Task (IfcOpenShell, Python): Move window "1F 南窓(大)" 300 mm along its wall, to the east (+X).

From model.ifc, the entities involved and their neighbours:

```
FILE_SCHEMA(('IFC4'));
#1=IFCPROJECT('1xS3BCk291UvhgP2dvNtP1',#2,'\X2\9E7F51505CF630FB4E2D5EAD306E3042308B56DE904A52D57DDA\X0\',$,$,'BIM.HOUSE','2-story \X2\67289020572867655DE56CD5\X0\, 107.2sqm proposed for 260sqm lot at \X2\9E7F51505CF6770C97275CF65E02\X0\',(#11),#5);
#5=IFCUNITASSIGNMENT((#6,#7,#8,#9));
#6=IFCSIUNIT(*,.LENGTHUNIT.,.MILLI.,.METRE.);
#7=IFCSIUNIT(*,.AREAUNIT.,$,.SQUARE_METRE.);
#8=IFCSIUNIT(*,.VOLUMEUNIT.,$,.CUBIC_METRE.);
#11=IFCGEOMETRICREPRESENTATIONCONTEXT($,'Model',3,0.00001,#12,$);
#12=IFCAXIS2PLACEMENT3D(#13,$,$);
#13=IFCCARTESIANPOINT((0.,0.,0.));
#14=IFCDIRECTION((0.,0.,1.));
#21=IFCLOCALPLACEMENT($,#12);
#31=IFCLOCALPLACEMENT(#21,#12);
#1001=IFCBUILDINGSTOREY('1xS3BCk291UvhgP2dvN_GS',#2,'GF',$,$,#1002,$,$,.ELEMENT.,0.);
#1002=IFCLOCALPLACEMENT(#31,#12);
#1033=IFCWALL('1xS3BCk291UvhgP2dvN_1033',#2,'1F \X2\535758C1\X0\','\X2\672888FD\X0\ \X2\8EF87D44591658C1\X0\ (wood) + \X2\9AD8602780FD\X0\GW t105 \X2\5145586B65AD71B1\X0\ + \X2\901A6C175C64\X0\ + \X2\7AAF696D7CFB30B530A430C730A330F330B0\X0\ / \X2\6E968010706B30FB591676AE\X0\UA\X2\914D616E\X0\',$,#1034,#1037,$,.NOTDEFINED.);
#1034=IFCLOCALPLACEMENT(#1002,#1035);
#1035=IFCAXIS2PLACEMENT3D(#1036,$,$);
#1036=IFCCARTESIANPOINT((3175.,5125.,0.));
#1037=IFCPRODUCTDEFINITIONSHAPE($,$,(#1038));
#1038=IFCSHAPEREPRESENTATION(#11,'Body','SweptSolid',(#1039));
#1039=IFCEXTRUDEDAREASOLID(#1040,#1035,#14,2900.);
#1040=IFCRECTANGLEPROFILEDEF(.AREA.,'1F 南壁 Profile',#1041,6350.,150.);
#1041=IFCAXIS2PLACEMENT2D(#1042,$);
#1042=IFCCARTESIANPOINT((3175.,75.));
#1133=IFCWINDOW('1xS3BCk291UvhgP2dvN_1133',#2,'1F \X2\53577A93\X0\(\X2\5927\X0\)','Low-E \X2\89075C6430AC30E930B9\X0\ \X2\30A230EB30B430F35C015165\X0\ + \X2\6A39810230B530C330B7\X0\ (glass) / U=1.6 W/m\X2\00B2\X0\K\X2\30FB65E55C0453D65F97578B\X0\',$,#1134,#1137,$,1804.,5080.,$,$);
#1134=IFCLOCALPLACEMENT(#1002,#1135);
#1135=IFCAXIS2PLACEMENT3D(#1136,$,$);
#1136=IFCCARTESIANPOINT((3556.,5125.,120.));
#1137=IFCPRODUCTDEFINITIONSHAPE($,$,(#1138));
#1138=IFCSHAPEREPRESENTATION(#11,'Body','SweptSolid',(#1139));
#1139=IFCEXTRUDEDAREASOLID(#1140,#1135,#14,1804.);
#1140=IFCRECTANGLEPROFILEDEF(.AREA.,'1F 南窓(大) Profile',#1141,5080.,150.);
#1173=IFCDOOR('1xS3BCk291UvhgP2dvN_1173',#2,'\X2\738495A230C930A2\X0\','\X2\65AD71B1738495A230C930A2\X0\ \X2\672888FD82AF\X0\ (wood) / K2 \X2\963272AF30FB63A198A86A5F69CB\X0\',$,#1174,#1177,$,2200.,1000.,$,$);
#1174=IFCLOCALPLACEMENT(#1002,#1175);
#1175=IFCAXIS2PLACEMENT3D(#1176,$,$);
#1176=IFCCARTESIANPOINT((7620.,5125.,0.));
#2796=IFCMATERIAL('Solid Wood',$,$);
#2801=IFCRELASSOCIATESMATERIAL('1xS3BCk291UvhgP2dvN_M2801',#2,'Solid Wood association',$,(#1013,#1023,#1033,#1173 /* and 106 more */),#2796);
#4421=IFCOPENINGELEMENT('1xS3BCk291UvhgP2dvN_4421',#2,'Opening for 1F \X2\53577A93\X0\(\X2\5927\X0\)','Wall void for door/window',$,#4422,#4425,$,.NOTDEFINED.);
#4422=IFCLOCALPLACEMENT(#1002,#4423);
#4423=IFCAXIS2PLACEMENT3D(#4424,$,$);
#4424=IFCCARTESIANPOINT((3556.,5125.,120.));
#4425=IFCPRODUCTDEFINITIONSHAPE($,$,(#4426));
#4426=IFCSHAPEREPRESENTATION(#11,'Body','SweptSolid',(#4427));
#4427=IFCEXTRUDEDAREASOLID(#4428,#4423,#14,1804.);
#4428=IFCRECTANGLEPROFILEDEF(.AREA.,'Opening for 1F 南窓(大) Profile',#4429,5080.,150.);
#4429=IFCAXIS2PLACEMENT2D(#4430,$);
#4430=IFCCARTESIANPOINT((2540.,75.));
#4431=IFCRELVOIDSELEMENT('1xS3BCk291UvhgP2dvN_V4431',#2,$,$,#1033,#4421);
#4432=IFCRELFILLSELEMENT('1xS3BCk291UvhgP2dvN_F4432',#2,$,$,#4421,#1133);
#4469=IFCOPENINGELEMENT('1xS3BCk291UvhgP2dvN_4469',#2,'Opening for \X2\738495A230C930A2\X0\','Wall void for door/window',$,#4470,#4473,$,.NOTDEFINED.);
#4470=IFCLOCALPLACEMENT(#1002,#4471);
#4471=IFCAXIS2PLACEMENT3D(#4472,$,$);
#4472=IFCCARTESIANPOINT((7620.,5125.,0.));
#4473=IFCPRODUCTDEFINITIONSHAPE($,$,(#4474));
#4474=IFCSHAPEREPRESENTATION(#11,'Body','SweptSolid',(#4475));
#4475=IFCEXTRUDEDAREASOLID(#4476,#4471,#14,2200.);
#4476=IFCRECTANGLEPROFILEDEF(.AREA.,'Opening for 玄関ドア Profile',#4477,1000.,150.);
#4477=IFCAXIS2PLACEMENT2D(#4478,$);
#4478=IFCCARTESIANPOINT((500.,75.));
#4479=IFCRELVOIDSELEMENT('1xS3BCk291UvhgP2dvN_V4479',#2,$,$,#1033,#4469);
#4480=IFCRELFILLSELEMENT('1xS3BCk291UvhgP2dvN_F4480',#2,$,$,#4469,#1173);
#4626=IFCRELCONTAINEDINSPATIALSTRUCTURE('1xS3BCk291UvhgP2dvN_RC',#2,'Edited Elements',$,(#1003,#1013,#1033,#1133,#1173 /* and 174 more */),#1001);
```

```python
import ifcopenshell
import ifcopenshell.api.geometry
import ifcopenshell.util.placement

model = ifcopenshell.open("model.ifc")

window = model.by_id(1133)
opening = window.FillsVoids[0].RelatingOpeningElement
wall = opening.VoidsElements[0].RelatingBuildingElement

wall_matrix = ifcopenshell.util.placement.get_local_placement(wall.ObjectPlacement)
shift = wall_matrix[:3, 0] * 300.0
before = ifcopenshell.util.placement.get_local_placement(window.ObjectPlacement)[:3, 3].copy()

# The window is not placed relative to its opening, so move both.
for product in (opening, window):
    matrix = ifcopenshell.util.placement.get_local_placement(product.ObjectPlacement)
    matrix[:3, 3] += shift
    ifcopenshell.api.geometry.edit_object_placement(model, product=product, matrix=matrix, is_si=False)

after = ifcopenshell.util.placement.get_local_placement(window.ObjectPlacement)[:3, 3]
print("window moved by", (after - before).round(3) + 0.0)

model.write("model_updated.ifc")
```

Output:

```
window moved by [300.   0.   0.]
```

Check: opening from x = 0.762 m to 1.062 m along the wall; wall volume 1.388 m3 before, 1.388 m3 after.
